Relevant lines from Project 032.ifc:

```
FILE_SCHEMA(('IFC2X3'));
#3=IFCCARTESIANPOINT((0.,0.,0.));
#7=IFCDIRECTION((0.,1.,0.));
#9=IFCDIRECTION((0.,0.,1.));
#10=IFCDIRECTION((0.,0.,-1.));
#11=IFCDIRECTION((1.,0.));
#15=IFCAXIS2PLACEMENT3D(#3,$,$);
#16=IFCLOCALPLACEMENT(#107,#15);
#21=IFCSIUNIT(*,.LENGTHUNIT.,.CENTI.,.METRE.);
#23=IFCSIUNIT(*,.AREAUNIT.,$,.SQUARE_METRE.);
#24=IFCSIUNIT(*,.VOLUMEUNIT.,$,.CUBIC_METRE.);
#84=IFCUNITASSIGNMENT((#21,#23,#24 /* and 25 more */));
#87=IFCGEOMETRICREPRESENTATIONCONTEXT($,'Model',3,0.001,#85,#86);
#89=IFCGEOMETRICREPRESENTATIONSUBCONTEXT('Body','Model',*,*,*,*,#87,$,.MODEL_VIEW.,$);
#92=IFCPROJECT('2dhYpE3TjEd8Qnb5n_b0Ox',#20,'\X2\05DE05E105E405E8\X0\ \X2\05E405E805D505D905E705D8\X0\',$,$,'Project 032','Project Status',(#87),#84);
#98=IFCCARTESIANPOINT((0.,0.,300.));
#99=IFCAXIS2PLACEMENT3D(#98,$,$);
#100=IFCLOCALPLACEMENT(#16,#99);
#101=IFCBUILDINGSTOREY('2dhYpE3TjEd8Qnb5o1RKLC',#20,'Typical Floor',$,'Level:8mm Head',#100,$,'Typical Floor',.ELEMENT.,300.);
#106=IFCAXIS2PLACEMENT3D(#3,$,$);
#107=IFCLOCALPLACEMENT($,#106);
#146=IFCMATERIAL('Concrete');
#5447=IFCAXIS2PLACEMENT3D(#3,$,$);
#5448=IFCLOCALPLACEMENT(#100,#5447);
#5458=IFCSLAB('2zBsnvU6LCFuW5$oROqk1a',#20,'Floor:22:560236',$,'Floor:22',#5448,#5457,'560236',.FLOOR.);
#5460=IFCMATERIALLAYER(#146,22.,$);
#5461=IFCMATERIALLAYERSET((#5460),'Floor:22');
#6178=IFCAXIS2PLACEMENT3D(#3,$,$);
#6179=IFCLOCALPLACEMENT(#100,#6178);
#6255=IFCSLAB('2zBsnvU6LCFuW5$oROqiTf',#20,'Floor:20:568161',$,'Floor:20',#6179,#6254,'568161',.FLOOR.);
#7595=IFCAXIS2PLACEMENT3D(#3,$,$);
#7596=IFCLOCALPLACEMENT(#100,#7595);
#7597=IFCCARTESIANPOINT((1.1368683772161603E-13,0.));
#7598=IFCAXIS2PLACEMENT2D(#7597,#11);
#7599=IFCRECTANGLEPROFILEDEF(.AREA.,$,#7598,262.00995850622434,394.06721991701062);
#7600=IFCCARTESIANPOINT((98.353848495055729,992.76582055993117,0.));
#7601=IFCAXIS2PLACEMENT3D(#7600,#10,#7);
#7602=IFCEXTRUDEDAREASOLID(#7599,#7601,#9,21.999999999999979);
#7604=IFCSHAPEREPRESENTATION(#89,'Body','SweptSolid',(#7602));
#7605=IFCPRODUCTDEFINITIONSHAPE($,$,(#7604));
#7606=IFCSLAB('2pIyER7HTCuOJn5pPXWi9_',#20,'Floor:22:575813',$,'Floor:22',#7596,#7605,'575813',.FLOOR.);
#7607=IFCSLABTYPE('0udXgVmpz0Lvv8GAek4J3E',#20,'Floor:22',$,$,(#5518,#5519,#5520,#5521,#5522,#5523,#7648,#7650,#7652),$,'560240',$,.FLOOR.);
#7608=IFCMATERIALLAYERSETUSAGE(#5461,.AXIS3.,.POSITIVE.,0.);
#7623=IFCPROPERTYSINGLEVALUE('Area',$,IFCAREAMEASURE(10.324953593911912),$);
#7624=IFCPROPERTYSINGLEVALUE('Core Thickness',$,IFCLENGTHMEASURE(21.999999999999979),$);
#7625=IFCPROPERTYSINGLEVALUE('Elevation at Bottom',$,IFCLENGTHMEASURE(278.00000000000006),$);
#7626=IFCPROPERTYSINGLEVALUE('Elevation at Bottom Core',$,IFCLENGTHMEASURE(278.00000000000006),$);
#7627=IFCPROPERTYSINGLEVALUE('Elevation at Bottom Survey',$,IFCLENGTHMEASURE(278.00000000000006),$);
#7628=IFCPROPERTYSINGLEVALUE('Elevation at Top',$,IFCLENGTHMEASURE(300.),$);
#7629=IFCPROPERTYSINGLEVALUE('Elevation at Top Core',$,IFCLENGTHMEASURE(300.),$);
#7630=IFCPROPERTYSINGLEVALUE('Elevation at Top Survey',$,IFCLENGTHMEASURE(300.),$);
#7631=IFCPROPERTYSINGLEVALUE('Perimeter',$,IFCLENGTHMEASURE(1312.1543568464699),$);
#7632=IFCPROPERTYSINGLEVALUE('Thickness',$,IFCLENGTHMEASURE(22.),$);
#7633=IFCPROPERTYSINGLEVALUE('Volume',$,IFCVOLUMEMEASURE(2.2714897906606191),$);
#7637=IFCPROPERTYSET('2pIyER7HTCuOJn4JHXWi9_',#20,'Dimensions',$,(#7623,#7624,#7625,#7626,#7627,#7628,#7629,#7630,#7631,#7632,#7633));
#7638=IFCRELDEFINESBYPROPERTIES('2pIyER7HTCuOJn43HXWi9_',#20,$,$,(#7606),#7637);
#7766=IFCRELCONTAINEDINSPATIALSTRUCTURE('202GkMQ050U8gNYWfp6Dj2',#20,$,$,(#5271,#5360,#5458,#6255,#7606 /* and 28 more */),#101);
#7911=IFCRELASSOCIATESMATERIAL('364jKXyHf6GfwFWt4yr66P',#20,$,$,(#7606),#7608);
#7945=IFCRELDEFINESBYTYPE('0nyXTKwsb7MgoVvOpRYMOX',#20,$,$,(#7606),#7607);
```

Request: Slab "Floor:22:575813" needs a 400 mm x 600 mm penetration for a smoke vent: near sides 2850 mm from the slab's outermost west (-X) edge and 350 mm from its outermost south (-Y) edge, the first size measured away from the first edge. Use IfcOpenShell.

```python
import numpy as np
import ifcopenshell
import ifcopenshell.api.feature
import ifcopenshell.api.geometry
import ifcopenshell.api.pset
import ifcopenshell.api.root
import ifcopenshell.geom
import ifcopenshell.util.element
import ifcopenshell.util.placement
import ifcopenshell.util.representation
import ifcopenshell.util.shape
import ifcopenshell.util.unit

model = ifcopenshell.open("Project 032.ifc")
unit_scale = ifcopenshell.util.unit.calculate_unit_scale(model)
area_scale = ifcopenshell.util.unit.calculate_unit_scale(model, "AREAUNIT")
volume_scale = ifcopenshell.util.unit.calculate_unit_scale(model, "VOLUMEUNIT")
settings = ifcopenshell.geom.settings()


def volume(element):
    """Net volume in cubic metres, openings subtracted."""
    shape = ifcopenshell.geom.create_shape(settings, element)
    return ifcopenshell.util.shape.get_volume(shape.geometry)


slab = model.by_guid("2pIyER7HTCuOJn5pPXWi9_")
before = volume(slab)

# Extent in the slab's own axes, in metres. The edges named are its -X and -Y sides.
slab_shape = ifcopenshell.geom.create_shape(settings, slab)
vertices = ifcopenshell.util.shape.get_vertices(slab_shape.geometry)
x_min, y_min, bottom = vertices.min(axis=0)
top = vertices[:, 2].max()

opening = ifcopenshell.api.root.create_entity(model, ifc_class="IfcOpeningElement", name="Smoke vent opening")
context = ifcopenshell.util.representation.get_context(model, "Model", "Body", "MODEL_VIEW")
width, depth = 0.4, 0.6
outline = [(0.0, 0.0), (width, 0.0), (width, depth), (0.0, depth), (0.0, 0.0)]
# Overshoot both faces by 50 mm so the cut is clean.
shape = ifcopenshell.api.geometry.add_slab_representation(
    model, context=context, depth=top - bottom + 0.1, polyline=outline
)
ifcopenshell.api.geometry.assign_representation(model, product=opening, representation=shape)

matrix = ifcopenshell.util.placement.get_local_placement(slab.ObjectPlacement)
matrix[:, 3] = matrix @ np.append(np.array([x_min + 2.85, y_min + 0.35, bottom - 0.05]) / unit_scale, 1.0)
ifcopenshell.api.geometry.edit_object_placement(model, product=opening, matrix=matrix, is_si=False)
ifcopenshell.api.feature.add_feature(model, feature=opening, element=slab)

after = volume(slab)

# Update the slab's stored quantities.
pset = model.by_id(ifcopenshell.util.element.get_pset(slab, "Dimensions", should_inherit=False)["id"])
ifcopenshell.api.pset.edit_pset(model, pset=pset, properties={
    "Area": model.create_entity("IfcAreaMeasure", after / (top - bottom) / area_scale),
    "Volume": model.create_entity("IfcVolumeMeasure", after / volume_scale),
})

print(f"slab volume {before:.3f} -> {after:.3f} m3")

model.write("Project 032-out.ifc")
```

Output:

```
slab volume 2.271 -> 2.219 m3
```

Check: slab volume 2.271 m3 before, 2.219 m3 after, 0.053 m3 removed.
